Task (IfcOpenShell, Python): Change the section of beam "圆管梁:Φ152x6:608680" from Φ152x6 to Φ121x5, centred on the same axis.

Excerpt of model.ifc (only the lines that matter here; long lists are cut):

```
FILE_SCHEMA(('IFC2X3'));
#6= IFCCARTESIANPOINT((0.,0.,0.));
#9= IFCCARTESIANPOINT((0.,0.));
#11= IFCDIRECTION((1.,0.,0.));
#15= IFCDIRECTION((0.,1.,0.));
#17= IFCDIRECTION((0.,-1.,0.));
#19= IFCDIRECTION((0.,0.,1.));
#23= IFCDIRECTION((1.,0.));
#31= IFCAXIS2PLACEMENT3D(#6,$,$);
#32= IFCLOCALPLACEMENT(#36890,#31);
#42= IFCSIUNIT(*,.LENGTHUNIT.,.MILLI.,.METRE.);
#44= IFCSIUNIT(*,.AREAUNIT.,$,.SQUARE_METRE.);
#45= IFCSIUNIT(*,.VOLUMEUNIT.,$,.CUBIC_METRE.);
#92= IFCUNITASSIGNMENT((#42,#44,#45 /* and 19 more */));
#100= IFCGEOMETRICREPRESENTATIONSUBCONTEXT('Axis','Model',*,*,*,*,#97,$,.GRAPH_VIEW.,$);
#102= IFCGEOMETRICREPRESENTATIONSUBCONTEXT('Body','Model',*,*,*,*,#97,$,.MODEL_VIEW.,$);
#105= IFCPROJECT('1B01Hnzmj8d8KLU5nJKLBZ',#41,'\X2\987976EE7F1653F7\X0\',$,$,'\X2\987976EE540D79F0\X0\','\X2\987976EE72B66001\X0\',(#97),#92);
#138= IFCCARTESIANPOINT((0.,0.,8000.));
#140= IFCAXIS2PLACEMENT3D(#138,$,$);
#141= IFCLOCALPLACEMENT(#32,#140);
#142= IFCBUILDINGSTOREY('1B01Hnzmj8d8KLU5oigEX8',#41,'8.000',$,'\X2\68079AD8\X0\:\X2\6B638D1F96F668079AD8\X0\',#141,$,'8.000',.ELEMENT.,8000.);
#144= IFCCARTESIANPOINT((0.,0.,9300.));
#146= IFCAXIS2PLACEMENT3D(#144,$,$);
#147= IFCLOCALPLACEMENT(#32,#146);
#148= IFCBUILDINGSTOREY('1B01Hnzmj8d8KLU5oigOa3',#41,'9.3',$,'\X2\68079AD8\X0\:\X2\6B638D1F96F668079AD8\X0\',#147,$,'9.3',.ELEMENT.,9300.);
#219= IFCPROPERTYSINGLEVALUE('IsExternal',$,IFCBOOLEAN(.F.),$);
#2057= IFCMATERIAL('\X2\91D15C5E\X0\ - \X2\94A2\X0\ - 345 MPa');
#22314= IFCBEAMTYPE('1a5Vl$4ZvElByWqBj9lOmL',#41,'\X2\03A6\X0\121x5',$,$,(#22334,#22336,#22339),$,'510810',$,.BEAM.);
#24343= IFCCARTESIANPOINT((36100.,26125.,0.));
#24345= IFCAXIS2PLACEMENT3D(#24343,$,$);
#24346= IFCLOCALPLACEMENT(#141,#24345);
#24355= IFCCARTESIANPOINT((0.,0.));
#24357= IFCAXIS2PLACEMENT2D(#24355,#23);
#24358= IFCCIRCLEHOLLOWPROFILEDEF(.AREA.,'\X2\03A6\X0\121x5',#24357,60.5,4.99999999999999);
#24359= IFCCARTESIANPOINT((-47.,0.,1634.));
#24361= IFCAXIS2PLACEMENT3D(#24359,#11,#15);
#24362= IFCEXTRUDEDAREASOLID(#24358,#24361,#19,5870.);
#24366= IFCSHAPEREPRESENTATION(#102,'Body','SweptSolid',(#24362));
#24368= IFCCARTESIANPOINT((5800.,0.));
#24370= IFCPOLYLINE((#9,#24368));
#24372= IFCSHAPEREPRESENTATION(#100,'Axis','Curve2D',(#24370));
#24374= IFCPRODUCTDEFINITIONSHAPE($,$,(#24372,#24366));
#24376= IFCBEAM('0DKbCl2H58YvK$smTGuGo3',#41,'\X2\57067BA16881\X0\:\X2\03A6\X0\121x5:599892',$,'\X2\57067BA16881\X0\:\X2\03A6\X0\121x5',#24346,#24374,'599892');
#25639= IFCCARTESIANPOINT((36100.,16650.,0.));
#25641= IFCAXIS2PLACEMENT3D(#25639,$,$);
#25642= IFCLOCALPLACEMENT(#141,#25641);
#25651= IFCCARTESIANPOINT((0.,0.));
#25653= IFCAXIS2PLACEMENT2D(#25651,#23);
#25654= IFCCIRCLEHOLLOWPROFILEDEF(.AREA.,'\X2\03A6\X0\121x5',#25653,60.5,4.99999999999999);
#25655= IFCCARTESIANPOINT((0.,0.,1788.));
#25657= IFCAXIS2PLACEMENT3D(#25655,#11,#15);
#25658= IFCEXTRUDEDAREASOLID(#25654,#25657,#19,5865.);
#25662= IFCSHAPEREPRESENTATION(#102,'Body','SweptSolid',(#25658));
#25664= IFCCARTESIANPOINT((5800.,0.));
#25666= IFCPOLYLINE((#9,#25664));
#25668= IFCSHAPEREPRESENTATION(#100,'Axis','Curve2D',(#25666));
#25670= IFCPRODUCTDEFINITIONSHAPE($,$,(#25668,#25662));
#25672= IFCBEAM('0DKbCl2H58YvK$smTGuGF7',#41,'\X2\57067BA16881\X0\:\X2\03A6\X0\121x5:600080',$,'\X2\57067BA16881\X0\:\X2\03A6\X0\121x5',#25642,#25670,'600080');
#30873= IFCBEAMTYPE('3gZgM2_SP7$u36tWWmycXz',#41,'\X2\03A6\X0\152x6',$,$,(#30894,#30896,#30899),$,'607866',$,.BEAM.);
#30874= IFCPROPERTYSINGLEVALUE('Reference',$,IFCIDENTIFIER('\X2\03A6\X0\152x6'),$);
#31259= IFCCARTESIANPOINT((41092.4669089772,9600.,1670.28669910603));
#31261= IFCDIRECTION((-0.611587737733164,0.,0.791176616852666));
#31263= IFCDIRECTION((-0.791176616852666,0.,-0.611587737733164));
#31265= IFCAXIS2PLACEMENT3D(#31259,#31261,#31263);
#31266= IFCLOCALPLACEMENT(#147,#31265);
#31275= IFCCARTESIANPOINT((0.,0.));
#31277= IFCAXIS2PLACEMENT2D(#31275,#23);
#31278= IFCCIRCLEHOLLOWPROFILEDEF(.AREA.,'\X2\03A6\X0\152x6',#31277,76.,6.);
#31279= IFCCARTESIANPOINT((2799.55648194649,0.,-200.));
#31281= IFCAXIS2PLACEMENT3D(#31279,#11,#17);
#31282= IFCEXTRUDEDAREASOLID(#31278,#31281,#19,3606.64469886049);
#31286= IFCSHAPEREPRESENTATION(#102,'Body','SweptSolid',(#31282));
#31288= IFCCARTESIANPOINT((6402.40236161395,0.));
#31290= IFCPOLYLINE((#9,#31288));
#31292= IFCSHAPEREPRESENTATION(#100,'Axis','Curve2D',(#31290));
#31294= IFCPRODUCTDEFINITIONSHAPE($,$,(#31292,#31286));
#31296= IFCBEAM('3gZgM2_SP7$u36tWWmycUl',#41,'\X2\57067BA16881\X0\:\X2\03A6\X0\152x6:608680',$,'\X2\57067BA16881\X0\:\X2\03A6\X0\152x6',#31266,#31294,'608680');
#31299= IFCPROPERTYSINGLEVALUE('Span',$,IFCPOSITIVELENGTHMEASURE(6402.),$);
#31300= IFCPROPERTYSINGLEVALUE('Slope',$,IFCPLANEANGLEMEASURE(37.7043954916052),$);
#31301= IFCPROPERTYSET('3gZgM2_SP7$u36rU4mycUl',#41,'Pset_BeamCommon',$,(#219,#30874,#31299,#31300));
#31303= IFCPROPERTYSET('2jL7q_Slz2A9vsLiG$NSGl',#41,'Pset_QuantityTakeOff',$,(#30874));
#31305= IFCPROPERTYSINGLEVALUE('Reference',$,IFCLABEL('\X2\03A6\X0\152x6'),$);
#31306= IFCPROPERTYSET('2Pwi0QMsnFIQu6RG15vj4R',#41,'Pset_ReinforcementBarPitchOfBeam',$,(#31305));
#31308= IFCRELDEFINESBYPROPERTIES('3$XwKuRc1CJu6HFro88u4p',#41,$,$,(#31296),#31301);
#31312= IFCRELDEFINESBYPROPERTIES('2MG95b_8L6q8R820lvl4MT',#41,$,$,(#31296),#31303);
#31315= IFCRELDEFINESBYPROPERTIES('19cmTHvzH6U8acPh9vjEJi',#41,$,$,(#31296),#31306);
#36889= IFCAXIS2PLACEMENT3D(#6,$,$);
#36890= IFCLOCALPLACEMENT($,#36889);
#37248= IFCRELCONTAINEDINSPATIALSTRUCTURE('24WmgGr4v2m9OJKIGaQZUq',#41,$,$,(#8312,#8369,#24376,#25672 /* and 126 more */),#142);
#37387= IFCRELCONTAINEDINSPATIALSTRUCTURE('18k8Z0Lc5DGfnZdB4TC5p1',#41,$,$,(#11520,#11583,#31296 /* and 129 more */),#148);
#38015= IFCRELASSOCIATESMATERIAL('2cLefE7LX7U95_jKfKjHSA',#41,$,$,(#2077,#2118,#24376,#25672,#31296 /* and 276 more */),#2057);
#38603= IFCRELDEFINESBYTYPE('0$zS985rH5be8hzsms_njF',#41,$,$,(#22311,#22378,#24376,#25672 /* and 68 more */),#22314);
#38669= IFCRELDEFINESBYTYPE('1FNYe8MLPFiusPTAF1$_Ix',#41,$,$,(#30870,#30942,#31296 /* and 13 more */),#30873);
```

```python
import ifcopenshell
import ifcopenshell.api.pset
import ifcopenshell.api.type
import ifcopenshell.util.element
import ifcopenshell.util.representation

model = ifcopenshell.open("model.ifc")

member = model.by_guid("3gZgM2_SP7$u36tWWmycUl")
source = next(p for p in model.by_type("IfcCircleHollowProfileDef") if p.ProfileName == "Φ121x5")

body = ifcopenshell.util.representation.get_representation(member, "Model", "Body")
solid = body.Items[0]
old_profile = solid.SweptArea

# Copy the section's sizes but keep this member's own profile position.
profile = ifcopenshell.util.element.copy(model, source)
profile.Position = old_profile.Position
solid.SweptArea = profile
if not model.get_total_inverses(old_profile):
    ifcopenshell.util.element.remove_deep2(model, old_profile)

new_type = model.by_id(22314)
ifcopenshell.api.type.assign_type(
    model, related_objects=[member], relating_type=new_type, should_map_representations=False
)
member.Name = member.Name.replace("Φ152x6", "Φ121x5")
member.ObjectType = "圆管梁:Φ121x5"
pset = model.by_id(ifcopenshell.util.element.get_pset(member, "Pset_BeamCommon", should_inherit=False)["id"])
ifcopenshell.api.pset.edit_pset(model, pset=pset, properties={"Reference": "Φ121x5"})
pset = model.by_id(ifcopenshell.util.element.get_pset(member, "Pset_QuantityTakeOff", should_inherit=False)["id"])
ifcopenshell.api.pset.edit_pset(model, pset=pset, properties={"Reference": "Φ121x5"})
pset = model.by_id(ifcopenshell.util.element.get_pset(member, "Pset_ReinforcementBarPitchOfBeam", should_inherit=False)["id"])
ifcopenshell.api.pset.edit_pset(model, pset=pset, properties={"Reference": "Φ121x5"})

print(solid.SweptArea)

model.write("model-out.ifc")
```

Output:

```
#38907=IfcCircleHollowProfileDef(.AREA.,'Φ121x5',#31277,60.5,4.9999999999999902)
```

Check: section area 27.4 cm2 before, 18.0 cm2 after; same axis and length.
